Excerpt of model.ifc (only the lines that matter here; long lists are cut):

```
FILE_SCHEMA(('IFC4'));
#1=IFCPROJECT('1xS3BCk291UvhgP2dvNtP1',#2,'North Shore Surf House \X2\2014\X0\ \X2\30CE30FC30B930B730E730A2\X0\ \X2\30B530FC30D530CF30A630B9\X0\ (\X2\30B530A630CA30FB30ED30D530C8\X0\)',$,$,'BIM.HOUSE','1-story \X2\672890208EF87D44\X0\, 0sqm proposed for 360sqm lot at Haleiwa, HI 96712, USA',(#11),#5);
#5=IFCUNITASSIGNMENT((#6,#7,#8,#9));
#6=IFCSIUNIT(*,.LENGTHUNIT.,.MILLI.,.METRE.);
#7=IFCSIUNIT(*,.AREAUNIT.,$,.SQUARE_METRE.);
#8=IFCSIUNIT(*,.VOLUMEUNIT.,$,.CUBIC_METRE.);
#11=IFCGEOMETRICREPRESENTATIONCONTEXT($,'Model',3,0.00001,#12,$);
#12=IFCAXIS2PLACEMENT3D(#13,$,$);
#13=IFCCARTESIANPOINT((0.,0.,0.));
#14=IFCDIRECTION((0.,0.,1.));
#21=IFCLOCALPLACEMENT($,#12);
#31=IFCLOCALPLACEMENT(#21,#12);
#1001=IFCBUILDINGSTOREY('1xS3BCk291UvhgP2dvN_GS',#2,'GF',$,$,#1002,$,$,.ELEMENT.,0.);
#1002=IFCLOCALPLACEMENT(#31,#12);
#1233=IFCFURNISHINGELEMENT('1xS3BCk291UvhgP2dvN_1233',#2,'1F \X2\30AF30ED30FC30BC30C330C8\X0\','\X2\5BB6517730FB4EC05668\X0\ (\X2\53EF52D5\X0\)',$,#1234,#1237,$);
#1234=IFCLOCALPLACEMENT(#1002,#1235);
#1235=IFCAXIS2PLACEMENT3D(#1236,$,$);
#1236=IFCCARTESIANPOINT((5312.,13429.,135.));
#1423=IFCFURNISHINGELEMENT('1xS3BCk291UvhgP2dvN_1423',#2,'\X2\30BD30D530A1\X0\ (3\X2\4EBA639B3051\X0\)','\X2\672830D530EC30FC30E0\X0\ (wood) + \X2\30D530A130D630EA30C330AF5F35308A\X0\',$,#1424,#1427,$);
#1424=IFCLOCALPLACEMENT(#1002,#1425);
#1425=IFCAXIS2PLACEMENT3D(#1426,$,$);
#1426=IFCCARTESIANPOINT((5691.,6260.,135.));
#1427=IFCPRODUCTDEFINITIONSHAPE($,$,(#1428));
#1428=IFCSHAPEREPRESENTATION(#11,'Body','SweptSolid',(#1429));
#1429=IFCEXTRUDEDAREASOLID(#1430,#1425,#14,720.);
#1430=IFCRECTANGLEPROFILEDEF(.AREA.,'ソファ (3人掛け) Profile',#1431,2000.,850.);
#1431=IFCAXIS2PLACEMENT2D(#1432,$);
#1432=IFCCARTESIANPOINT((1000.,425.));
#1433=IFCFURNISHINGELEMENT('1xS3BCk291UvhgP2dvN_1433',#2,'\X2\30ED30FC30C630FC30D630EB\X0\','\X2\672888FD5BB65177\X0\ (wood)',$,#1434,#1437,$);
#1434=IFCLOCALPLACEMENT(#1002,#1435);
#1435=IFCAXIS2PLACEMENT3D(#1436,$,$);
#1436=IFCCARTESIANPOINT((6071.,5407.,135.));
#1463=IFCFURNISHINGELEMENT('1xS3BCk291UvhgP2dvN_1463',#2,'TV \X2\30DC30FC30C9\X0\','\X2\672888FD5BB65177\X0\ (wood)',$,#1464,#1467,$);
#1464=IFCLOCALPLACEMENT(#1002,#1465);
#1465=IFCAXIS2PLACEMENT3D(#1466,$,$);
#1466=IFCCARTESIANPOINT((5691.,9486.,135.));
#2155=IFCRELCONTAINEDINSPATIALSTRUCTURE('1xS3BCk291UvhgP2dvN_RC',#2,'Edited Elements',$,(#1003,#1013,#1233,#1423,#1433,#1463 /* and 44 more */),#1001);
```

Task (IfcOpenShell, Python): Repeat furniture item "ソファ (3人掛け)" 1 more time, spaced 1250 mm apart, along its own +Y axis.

```python
import ifcopenshell
import ifcopenshell.api.geometry
import ifcopenshell.api.root
import ifcopenshell.util.element
import ifcopenshell.util.placement
import ifcopenshell.util.unit

model = ifcopenshell.open("model.ifc")
unit_scale = ifcopenshell.util.unit.calculate_unit_scale(model)


def reuse_history(source, copy):
    """copy_class also copies each property set's owner history, people and application; keep the originals."""
    for rel in copy.IsDefinedBy:
        if rel.is_a("IfcRelDefinesByProperties") and (history := rel.RelatingPropertyDefinition.OwnerHistory):
            rel.RelatingPropertyDefinition.OwnerHistory = source.OwnerHistory
            ifcopenshell.util.element.remove_deep2(model, history)


source = model.by_id(1423)
base = ifcopenshell.util.placement.get_local_placement(source.ObjectPlacement)
step = base[:3, 1] * 1.25 / unit_scale

for i in range(1, 2):
    copy = ifcopenshell.api.root.copy_class(model, product=source)
    copy.Representation = ifcopenshell.util.element.copy_deep(
        model, source.Representation, exclude=["IfcGeometricRepresentationContext", "IfcRepresentationMap"]
    )
    reuse_history(source, copy)
    matrix = base.copy()
    matrix[:3, 3] += i * step
    print("added at", matrix[:3, 3].round(3) + 0.0)
    ifcopenshell.api.geometry.edit_object_placement(model, product=copy, matrix=matrix, is_si=False)

model.write("model_v2.ifc")
```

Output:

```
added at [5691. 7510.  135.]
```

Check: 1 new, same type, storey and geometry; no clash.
